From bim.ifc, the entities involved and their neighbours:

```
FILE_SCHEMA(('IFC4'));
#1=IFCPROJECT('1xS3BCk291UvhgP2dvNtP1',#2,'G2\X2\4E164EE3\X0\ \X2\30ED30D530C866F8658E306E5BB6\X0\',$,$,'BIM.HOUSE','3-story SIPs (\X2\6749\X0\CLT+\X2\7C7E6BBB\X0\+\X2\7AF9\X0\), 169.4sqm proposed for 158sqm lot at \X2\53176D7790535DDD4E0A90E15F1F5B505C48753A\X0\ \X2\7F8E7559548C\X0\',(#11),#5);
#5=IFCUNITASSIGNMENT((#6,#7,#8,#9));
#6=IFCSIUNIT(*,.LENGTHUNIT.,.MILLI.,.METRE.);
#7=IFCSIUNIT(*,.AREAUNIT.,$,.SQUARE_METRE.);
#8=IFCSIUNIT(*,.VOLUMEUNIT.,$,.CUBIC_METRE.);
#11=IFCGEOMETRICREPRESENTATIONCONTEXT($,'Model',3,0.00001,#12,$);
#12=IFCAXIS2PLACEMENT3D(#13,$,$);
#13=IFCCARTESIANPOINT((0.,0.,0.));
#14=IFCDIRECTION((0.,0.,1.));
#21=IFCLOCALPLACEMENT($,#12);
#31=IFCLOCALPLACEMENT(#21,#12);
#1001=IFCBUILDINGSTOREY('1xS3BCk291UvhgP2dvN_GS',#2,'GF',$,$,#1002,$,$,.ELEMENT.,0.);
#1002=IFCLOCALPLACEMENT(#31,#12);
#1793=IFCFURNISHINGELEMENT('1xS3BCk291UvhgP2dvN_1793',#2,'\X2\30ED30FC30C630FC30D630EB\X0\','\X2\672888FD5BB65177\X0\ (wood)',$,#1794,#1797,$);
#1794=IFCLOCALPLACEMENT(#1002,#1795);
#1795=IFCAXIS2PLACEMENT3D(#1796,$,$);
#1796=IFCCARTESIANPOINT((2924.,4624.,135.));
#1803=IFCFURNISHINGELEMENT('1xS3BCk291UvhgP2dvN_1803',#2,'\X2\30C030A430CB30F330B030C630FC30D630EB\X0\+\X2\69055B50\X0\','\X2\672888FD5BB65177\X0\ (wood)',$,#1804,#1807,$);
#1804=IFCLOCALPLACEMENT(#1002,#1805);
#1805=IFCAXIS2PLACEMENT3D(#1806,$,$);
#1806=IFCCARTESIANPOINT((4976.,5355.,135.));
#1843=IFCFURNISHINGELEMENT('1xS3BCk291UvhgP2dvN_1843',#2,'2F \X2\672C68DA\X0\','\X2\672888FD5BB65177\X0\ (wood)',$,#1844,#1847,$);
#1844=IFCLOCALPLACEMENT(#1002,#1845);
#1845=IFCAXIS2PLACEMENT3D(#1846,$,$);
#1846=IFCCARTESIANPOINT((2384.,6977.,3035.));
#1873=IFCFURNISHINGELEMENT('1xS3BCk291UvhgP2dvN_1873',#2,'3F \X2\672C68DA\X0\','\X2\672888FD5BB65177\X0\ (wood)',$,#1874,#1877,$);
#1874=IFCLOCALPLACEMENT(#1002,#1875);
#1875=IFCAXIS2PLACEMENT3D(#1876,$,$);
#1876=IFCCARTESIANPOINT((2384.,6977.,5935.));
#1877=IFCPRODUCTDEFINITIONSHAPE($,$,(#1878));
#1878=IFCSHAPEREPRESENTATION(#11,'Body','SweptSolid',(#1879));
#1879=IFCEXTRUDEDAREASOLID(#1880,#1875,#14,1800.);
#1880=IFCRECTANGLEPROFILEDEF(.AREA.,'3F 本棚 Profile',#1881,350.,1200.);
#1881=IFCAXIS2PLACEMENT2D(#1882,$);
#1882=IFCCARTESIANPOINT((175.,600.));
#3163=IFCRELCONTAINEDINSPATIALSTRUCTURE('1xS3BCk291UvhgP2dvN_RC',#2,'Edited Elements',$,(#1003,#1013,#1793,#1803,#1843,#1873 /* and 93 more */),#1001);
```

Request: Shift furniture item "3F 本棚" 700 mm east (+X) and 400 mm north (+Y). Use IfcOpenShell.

```python
import ifcopenshell
import ifcopenshell.api.geometry
import ifcopenshell.util.placement
import ifcopenshell.util.unit

model = ifcopenshell.open("bim.ifc")
unit_scale = ifcopenshell.util.unit.calculate_unit_scale(model)

item = model.by_guid("1xS3BCk291UvhgP2dvN_1873")
matrix = ifcopenshell.util.placement.get_local_placement(item.ObjectPlacement)
matrix[0, 3] += 0.7 / unit_scale
matrix[1, 3] += 0.4 / unit_scale
ifcopenshell.api.geometry.edit_object_placement(model, product=item, matrix=matrix, is_si=False)

print(ifcopenshell.util.placement.get_local_placement(item.ObjectPlacement).round(3) + 0.0)

model.write("bim_edited.ifc")
```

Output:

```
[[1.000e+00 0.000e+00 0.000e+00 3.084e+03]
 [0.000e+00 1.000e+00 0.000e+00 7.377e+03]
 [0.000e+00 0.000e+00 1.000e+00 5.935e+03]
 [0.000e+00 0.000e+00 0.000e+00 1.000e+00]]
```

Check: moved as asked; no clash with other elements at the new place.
